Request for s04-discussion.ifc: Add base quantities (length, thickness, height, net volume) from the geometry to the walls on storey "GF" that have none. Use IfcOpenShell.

First a look at what the model holds.

```python
import ifcopenshell
import ifcopenshell.util.element
import ifcopenshell.util.unit

model = ifcopenshell.open("s04-discussion.ifc")
print(model.schema)
for unit_type in ("LENGTHUNIT", "AREAUNIT", "VOLUMEUNIT"):
    print(unit_type, ifcopenshell.util.unit.calculate_unit_scale(model, unit_type))
storey = next(s for s in model.by_type("IfcBuildingStorey") if s.Name == "GF")
walls = [e for e in ifcopenshell.util.element.get_decomposition(storey) if e.is_a("IfcWall")]
for e in sorted(walls, key=lambda e: e.id()):
    print(e.id(), e.is_a(), e.Name, list(ifcopenshell.util.element.get_psets(e, qtos_only=True)), sep=" | ")
```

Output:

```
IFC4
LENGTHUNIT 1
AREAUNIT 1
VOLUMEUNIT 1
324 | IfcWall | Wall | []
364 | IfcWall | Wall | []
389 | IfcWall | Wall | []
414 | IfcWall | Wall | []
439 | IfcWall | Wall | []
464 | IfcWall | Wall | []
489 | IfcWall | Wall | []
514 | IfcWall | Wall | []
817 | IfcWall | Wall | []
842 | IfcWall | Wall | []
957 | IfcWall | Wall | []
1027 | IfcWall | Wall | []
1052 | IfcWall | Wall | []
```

```python
import ifcopenshell
import ifcopenshell.api.pset
import ifcopenshell.geom
import ifcopenshell.util.element
import ifcopenshell.util.shape
import ifcopenshell.util.unit

model = ifcopenshell.open("s04-discussion.ifc")
unit_scale = ifcopenshell.util.unit.calculate_unit_scale(model)
volume_scale = ifcopenshell.util.unit.calculate_unit_scale(model, "VOLUMEUNIT")
settings = ifcopenshell.geom.settings()

storey = next(s for s in model.by_type("IfcBuildingStorey") if s.Name == "GF")
walls = [e for e in ifcopenshell.util.element.get_decomposition(storey) if e.is_a("IfcWall")]

for e in sorted(walls, key=lambda e: e.id()):
    if ifcopenshell.util.element.get_psets(e, qtos_only=True, should_inherit=False):
        continue
    # Geometry comes back in metres, in the element's own axes.
    shape = ifcopenshell.geom.create_shape(settings, e)
    values = {
        "Length": ifcopenshell.util.shape.get_x(shape.geometry) / unit_scale,
        "Width": ifcopenshell.util.shape.get_y(shape.geometry) / unit_scale,
        "Height": ifcopenshell.util.shape.get_z(shape.geometry) / unit_scale,
        "NetVolume": ifcopenshell.util.shape.get_volume(shape.geometry) / volume_scale,
    }
    qto = ifcopenshell.api.pset.add_qto(model, product=e, name="Qto_WallBaseQuantities")
    ifcopenshell.api.pset.edit_qto(model, qto=qto, properties=values)
    print(e.id(), {k: round(v, 3) for k, v in values.items()})

model.write("s04-discussion_rev.ifc")
```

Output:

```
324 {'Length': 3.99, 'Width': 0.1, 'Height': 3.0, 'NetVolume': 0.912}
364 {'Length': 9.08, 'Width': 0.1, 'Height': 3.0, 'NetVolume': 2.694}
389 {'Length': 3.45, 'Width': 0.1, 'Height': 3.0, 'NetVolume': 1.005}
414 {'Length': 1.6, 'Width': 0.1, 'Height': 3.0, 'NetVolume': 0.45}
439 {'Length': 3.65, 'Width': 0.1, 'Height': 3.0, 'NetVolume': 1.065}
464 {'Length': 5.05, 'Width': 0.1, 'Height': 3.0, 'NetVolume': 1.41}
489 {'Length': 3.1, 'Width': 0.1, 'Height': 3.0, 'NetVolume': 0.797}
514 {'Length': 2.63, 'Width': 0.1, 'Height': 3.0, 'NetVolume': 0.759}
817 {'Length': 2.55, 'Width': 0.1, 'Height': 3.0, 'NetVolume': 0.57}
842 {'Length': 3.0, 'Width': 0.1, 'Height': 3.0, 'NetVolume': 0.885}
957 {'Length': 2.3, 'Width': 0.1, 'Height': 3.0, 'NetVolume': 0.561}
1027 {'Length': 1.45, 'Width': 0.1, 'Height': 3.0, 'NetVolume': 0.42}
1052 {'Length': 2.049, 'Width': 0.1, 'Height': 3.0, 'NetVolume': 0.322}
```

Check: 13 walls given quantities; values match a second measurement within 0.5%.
